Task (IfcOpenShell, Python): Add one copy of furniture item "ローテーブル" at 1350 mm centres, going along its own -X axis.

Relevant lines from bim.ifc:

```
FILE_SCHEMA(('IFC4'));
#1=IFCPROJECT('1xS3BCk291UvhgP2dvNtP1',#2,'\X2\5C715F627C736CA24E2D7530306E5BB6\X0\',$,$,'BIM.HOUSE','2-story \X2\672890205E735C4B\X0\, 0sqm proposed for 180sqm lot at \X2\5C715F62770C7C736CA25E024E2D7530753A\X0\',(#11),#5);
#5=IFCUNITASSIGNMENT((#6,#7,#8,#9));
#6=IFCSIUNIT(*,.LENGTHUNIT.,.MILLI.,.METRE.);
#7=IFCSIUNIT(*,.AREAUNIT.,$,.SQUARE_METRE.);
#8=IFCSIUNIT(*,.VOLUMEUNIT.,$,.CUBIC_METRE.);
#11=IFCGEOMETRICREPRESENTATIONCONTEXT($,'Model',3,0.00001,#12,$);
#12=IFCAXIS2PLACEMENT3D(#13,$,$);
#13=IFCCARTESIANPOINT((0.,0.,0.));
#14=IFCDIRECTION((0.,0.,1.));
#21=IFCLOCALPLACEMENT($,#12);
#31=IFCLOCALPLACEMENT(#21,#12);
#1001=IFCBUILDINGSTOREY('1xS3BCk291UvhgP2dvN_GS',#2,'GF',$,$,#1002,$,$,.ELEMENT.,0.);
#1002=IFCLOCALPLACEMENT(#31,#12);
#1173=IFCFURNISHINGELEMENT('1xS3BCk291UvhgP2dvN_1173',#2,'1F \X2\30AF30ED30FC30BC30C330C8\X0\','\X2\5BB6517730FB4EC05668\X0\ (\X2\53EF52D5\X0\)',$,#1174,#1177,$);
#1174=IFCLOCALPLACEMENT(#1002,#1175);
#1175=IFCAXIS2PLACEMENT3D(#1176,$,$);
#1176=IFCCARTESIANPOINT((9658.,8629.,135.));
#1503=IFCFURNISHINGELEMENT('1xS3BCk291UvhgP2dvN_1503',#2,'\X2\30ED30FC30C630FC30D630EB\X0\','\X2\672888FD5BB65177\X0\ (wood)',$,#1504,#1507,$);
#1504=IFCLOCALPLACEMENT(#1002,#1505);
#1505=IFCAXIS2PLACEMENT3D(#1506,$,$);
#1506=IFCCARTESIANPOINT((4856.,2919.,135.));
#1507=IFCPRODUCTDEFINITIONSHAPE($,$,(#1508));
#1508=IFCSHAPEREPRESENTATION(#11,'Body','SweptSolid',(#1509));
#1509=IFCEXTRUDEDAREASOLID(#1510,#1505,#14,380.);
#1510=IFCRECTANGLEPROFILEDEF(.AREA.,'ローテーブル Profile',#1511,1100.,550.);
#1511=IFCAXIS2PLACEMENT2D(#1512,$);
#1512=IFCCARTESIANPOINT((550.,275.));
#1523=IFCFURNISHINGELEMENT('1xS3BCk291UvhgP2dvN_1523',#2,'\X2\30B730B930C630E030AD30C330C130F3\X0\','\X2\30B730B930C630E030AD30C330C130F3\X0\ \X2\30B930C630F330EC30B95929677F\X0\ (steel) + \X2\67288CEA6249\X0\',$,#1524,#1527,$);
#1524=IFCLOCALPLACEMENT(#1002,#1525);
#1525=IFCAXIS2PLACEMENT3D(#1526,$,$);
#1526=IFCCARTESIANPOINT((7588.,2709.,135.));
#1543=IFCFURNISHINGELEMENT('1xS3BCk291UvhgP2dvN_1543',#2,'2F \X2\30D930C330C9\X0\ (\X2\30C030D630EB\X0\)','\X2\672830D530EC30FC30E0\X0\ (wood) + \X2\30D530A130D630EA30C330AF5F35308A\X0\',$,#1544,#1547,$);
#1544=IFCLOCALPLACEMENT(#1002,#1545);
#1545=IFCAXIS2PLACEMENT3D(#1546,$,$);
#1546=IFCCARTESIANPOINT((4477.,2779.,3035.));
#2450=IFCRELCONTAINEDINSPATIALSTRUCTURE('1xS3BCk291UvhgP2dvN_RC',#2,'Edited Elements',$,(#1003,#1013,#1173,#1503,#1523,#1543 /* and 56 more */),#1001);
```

```python
import ifcopenshell
import ifcopenshell.api.geometry
import ifcopenshell.api.root
import ifcopenshell.util.element
import ifcopenshell.util.placement
import ifcopenshell.util.unit

model = ifcopenshell.open("bim.ifc")
unit_scale = ifcopenshell.util.unit.calculate_unit_scale(model)


def reuse_history(source, copy):
    """copy_class also copies each property set's owner history, people and application; keep the originals."""
    for rel in copy.IsDefinedBy:
        if rel.is_a("IfcRelDefinesByProperties") and (history := rel.RelatingPropertyDefinition.OwnerHistory):
            rel.RelatingPropertyDefinition.OwnerHistory = source.OwnerHistory
            ifcopenshell.util.element.remove_deep2(model, history)


source = model.by_guid("1xS3BCk291UvhgP2dvN_1503")
base = ifcopenshell.util.placement.get_local_placement(source.ObjectPlacement)
step = -base[:3, 0] * 1.35 / unit_scale

for i in range(1, 2):
    copy = ifcopenshell.api.root.copy_class(model, product=source)
    copy.Representation = ifcopenshell.util.element.copy_deep(
        model, source.Representation, exclude=["IfcGeometricRepresentationContext", "IfcRepresentationMap"]
    )
    reuse_history(source, copy)
    matrix = base.copy()
    matrix[:3, 3] += i * step
    print("added at", matrix[:3, 3].round(3) + 0.0)
    ifcopenshell.api.geometry.edit_object_placement(model, product=copy, matrix=matrix, is_si=False)

model.write("bim_v2.ifc")
```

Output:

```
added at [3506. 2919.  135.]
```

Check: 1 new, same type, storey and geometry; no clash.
